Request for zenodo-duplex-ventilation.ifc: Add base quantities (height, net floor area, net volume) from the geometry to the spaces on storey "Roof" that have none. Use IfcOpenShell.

First a look at what the model holds.

```python
import ifcopenshell
import ifcopenshell.util.element
import ifcopenshell.util.unit

model = ifcopenshell.open("zenodo-duplex-ventilation.ifc")
print(model.schema)
for unit_type in ("LENGTHUNIT", "AREAUNIT", "VOLUMEUNIT"):
    print(unit_type, ifcopenshell.util.unit.calculate_unit_scale(model, unit_type))
storey = next(s for s in model.by_type("IfcBuildingStorey") if s.Name == "Roof")
spaces = [e for e in ifcopenshell.util.element.get_decomposition(storey) if e.is_a("IfcSpace")]
for e in sorted(spaces, key=lambda e: e.id()):
    print(e.id(), e.is_a(), e.Name, list(ifcopenshell.util.element.get_psets(e, qtos_only=True)), sep=" | ")
```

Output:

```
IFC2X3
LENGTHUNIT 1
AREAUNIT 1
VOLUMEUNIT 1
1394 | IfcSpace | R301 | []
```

```python
import ifcopenshell
import ifcopenshell.api.pset
import ifcopenshell.geom
import ifcopenshell.util.element
import ifcopenshell.util.shape
import ifcopenshell.util.unit

model = ifcopenshell.open("zenodo-duplex-ventilation.ifc")
unit_scale = ifcopenshell.util.unit.calculate_unit_scale(model)
area_scale = ifcopenshell.util.unit.calculate_unit_scale(model, "AREAUNIT")
volume_scale = ifcopenshell.util.unit.calculate_unit_scale(model, "VOLUMEUNIT")
settings = ifcopenshell.geom.settings()

storey = next(s for s in model.by_type("IfcBuildingStorey") if s.Name == "Roof")
spaces = [e for e in ifcopenshell.util.element.get_decomposition(storey) if e.is_a("IfcSpace")]

for e in sorted(spaces, key=lambda e: e.id()):
    if ifcopenshell.util.element.get_psets(e, qtos_only=True, should_inherit=False):
        continue
    # Geometry comes back in metres, in the element's own axes.
    shape = ifcopenshell.geom.create_shape(settings, e)
    values = {
        "Height": ifcopenshell.util.shape.get_z(shape.geometry) / unit_scale,
        "NetFloorArea": ifcopenshell.util.shape.get_footprint_area(shape.geometry) / area_scale,
        "NetVolume": ifcopenshell.util.shape.get_volume(shape.geometry) / volume_scale,
    }
    qto = ifcopenshell.api.pset.add_qto(model, product=e, name="BaseQuantities")
    ifcopenshell.api.pset.edit_qto(model, qto=qto, properties=values)
    print(e.id(), {k: round(v, 3) for k, v in values.items()})

model.write("zenodo-duplex-ventilation-out.ifc")
```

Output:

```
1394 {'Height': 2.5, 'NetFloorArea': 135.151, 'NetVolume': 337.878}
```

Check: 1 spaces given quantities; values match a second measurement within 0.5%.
